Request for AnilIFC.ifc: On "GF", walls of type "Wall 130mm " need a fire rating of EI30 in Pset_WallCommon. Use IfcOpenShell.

First a look at what the model holds.

```python
import ifcopenshell
import ifcopenshell.util.element

model = ifcopenshell.open("AnilIFC.ifc")
print(model.schema)
storey = next(s for s in model.by_type("IfcBuildingStorey") if s.Name == "GF")
walls = [e for e in ifcopenshell.util.element.get_decomposition(storey) if e.is_a("IfcWall")]
seen = {}
for e in walls:
    element_type = ifcopenshell.util.element.get_type(e)
    key = (element_type.Name if element_type != e and element_type else None, ifcopenshell.util.element.get_pset(e, "Pset_WallCommon", "FireRating"))
    seen[key] = seen.get(key, 0) + 1
for (name, value), count in sorted(seen.items(), key=str):
    print(count, "x", name, "|", value)
```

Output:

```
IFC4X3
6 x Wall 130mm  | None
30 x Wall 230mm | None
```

```python
import ifcopenshell
import ifcopenshell.api.pset
import ifcopenshell.util.element

model = ifcopenshell.open("AnilIFC.ifc")

storey = next(s for s in model.by_type("IfcBuildingStorey") if s.Name == "GF")
walls = [e for e in ifcopenshell.util.element.get_decomposition(storey) if e.is_a("IfcWall")]

count = 0
for e in walls:
    element_type = ifcopenshell.util.element.get_type(e)
    if element_type in (None, e) or element_type.Name != "Wall 130mm ":
        continue
    # add_pset returns the element's existing set when there is one.
    pset = ifcopenshell.api.pset.add_pset(model, product=e, name="Pset_WallCommon")
    ifcopenshell.api.pset.edit_pset(model, pset=pset, properties={"FireRating": "EI30"})
    count += 1

print(count, "walls updated")

model.write("AnilIFC_rev.ifc")
```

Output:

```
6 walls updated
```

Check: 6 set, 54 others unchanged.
